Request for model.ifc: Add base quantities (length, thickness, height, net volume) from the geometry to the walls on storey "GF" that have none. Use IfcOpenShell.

First a look at what the model holds.

```python
import ifcopenshell
import ifcopenshell.util.element
import ifcopenshell.util.unit

model = ifcopenshell.open("model.ifc")
print(model.schema)
for unit_type in ("LENGTHUNIT", "AREAUNIT", "VOLUMEUNIT"):
    print(unit_type, ifcopenshell.util.unit.calculate_unit_scale(model, unit_type))
storey = next(s for s in model.by_type("IfcBuildingStorey") if s.Name == "GF")
walls = [e for e in ifcopenshell.util.element.get_decomposition(storey) if e.is_a("IfcWall")]
for e in sorted(walls, key=lambda e: e.id()):
    print(e.id(), e.is_a(), e.Name, list(ifcopenshell.util.element.get_psets(e, qtos_only=True)), sep=" | ")
```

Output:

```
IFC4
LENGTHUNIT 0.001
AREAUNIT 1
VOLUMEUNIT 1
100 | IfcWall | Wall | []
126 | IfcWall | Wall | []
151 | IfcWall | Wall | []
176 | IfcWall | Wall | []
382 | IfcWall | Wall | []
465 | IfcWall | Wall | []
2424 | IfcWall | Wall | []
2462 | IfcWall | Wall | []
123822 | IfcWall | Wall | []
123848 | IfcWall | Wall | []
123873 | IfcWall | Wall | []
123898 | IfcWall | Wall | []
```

```python
import ifcopenshell
import ifcopenshell.api.pset
import ifcopenshell.geom
import ifcopenshell.util.element
import ifcopenshell.util.shape
import ifcopenshell.util.unit

model = ifcopenshell.open("model.ifc")
unit_scale = ifcopenshell.util.unit.calculate_unit_scale(model)
volume_scale = ifcopenshell.util.unit.calculate_unit_scale(model, "VOLUMEUNIT")
settings = ifcopenshell.geom.settings()

storey = next(s for s in model.by_type("IfcBuildingStorey") if s.Name == "GF")
walls = [e for e in ifcopenshell.util.element.get_decomposition(storey) if e.is_a("IfcWall")]

for e in sorted(walls, key=lambda e: e.id()):
    if ifcopenshell.util.element.get_psets(e, qtos_only=True, should_inherit=False):
        continue
    # Geometry comes back in metres, in the element's own axes.
    shape = ifcopenshell.geom.create_shape(settings, e)
    values = {
        "Length": ifcopenshell.util.shape.get_x(shape.geometry) / unit_scale,
        "Width": ifcopenshell.util.shape.get_y(shape.geometry) / unit_scale,
        "Height": ifcopenshell.util.shape.get_z(shape.geometry) / unit_scale,
        "NetVolume": ifcopenshell.util.shape.get_volume(shape.geometry) / volume_scale,
    }
    qto = ifcopenshell.api.pset.add_qto(model, product=e, name="Qto_WallBaseQuantities")
    ifcopenshell.api.pset.edit_qto(model, qto=qto, properties=values)
    print(e.id(), {k: round(v, 3) for k, v in values.items()})

model.write("model_edited.ifc")
```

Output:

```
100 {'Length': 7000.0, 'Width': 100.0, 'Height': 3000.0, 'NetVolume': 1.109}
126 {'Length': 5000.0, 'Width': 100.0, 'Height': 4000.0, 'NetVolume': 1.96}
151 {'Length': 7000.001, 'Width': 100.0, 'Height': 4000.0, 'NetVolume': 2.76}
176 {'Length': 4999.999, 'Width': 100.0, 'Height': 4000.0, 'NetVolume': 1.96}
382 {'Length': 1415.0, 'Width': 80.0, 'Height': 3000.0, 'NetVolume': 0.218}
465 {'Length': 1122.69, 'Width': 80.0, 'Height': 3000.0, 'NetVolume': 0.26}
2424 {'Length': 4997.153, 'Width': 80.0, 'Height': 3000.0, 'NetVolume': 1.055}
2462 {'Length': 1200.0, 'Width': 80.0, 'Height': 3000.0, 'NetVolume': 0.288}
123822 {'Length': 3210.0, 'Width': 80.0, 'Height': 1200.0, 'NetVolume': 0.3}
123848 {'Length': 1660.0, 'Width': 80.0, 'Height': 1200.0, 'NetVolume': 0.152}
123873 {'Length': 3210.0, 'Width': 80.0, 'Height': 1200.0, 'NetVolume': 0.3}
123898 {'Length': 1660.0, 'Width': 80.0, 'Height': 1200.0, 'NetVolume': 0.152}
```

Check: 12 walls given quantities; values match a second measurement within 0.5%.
